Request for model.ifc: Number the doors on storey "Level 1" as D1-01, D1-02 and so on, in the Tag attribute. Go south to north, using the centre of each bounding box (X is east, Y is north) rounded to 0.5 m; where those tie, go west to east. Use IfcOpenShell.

First a look at what the model holds.

```python
import ifcopenshell
import ifcopenshell.util.element
import ifcopenshell.util.placement

model = ifcopenshell.open("model.ifc")
print(model.schema)
storey = next(s for s in model.by_type("IfcBuildingStorey") if s.Name == "Level 1")
doors = [e for e in ifcopenshell.util.element.get_decomposition(storey) if e.is_a("IfcDoor")]
for e in sorted(doors, key=lambda e: e.id()):
    origin = ifcopenshell.util.placement.get_local_placement(e.ObjectPlacement)[:3, 3]
    print(e.id(), e.Tag, e.Name, origin.round(2) + 0.0, sep=" | ")
```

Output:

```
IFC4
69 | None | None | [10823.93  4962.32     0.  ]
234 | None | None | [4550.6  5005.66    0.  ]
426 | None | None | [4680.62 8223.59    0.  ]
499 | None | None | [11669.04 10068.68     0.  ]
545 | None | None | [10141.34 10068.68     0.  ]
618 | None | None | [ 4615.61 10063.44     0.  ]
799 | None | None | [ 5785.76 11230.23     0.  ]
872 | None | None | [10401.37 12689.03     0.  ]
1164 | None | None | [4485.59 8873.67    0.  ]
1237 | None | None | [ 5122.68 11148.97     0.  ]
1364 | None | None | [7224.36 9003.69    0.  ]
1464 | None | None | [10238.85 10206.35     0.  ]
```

```python
import ifcopenshell
import ifcopenshell.geom
import ifcopenshell.util.element
import ifcopenshell.util.shape

model = ifcopenshell.open("model.ifc")
settings = ifcopenshell.geom.settings()
settings.set("use-world-coords", True)


def centre(element):
    shape = ifcopenshell.geom.create_shape(settings, element)
    return ifcopenshell.util.shape.get_bbox_centroid(shape.geometry)


storey = next(s for s in model.by_type("IfcBuildingStorey") if s.Name == "Level 1")
doors = [e for e in ifcopenshell.util.element.get_decomposition(storey) if e.is_a("IfcDoor")]

# Insertion points can sit at a corner or the storey origin, so sort by the geometry (in metres).
centres = {e: centre(e) for e in doors}
doors.sort(key=lambda e: (round(centres[e][1] / 0.5), centres[e][0]))

for i, e in enumerate(doors, start=1):
    number = f"D1-{i:02d}"
    e.Tag = number
    print(e.id(), number)

model.write("model_updated.ifc")
```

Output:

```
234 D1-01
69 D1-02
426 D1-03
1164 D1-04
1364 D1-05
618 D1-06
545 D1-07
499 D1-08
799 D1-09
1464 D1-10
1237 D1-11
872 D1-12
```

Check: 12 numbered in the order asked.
